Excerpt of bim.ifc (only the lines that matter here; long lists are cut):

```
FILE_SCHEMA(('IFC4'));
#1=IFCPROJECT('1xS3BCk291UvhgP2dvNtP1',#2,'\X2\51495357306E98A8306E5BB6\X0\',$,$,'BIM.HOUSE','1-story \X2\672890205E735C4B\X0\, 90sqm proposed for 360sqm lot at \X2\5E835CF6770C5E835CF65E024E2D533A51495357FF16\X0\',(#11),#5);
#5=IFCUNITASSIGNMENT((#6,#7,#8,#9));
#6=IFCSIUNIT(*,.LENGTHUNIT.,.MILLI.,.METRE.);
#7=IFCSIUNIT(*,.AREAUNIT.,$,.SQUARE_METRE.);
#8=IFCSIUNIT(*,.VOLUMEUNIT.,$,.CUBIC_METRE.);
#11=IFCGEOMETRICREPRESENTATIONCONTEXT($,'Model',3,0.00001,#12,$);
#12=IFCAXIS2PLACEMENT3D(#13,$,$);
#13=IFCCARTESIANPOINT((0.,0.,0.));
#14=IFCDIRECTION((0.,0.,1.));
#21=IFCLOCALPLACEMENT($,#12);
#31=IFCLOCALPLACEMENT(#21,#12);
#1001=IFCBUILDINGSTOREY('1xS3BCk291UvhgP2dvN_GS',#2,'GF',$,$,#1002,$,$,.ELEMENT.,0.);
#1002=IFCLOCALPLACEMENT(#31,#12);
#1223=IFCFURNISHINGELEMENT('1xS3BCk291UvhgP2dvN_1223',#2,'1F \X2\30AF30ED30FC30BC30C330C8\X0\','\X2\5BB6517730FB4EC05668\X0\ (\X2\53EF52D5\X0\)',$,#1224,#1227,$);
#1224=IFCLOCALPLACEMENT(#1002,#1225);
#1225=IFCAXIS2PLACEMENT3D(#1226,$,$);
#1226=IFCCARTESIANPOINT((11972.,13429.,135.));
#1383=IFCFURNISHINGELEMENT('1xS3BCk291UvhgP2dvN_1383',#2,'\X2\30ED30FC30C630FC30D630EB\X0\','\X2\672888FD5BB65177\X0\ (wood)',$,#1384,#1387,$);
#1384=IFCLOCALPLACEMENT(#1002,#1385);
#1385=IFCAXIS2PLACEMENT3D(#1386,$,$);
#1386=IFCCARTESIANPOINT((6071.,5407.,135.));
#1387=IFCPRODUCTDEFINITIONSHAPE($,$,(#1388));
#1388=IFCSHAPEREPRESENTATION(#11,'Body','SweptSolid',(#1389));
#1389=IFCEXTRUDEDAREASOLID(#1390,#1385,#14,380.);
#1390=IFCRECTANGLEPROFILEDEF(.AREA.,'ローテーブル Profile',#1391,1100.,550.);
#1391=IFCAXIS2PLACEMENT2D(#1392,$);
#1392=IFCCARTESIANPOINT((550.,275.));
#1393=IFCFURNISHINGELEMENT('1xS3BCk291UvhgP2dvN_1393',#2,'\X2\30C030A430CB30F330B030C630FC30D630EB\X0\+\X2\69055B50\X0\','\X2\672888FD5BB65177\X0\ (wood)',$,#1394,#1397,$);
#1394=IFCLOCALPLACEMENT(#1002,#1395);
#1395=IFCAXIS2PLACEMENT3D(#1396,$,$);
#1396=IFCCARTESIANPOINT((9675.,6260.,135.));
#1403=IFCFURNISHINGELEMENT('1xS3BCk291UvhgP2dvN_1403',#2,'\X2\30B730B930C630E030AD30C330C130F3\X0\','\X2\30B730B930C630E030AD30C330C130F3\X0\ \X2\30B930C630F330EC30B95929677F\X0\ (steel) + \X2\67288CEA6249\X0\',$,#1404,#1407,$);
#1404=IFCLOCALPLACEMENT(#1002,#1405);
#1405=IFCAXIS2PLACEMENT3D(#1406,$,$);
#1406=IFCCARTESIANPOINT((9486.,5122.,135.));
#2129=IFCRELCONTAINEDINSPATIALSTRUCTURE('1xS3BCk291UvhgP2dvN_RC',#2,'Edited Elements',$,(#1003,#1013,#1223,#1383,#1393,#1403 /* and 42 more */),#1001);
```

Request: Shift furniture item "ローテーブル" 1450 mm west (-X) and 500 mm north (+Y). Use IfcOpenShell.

```python
import ifcopenshell
import ifcopenshell.api.geometry
import ifcopenshell.util.placement

model = ifcopenshell.open("bim.ifc")

item = model.by_guid("1xS3BCk291UvhgP2dvN_1383")
matrix = ifcopenshell.util.placement.get_local_placement(item.ObjectPlacement)
matrix[0, 3] -= 1450.0
matrix[1, 3] += 500.0
ifcopenshell.api.geometry.edit_object_placement(model, product=item, matrix=matrix, is_si=False)

print(ifcopenshell.util.placement.get_local_placement(item.ObjectPlacement).round(3) + 0.0)

model.write("bim_rev.ifc")
```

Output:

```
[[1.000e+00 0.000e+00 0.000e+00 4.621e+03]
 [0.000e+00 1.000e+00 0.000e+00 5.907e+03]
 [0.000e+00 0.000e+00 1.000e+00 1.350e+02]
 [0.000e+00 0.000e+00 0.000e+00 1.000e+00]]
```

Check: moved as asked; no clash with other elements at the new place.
